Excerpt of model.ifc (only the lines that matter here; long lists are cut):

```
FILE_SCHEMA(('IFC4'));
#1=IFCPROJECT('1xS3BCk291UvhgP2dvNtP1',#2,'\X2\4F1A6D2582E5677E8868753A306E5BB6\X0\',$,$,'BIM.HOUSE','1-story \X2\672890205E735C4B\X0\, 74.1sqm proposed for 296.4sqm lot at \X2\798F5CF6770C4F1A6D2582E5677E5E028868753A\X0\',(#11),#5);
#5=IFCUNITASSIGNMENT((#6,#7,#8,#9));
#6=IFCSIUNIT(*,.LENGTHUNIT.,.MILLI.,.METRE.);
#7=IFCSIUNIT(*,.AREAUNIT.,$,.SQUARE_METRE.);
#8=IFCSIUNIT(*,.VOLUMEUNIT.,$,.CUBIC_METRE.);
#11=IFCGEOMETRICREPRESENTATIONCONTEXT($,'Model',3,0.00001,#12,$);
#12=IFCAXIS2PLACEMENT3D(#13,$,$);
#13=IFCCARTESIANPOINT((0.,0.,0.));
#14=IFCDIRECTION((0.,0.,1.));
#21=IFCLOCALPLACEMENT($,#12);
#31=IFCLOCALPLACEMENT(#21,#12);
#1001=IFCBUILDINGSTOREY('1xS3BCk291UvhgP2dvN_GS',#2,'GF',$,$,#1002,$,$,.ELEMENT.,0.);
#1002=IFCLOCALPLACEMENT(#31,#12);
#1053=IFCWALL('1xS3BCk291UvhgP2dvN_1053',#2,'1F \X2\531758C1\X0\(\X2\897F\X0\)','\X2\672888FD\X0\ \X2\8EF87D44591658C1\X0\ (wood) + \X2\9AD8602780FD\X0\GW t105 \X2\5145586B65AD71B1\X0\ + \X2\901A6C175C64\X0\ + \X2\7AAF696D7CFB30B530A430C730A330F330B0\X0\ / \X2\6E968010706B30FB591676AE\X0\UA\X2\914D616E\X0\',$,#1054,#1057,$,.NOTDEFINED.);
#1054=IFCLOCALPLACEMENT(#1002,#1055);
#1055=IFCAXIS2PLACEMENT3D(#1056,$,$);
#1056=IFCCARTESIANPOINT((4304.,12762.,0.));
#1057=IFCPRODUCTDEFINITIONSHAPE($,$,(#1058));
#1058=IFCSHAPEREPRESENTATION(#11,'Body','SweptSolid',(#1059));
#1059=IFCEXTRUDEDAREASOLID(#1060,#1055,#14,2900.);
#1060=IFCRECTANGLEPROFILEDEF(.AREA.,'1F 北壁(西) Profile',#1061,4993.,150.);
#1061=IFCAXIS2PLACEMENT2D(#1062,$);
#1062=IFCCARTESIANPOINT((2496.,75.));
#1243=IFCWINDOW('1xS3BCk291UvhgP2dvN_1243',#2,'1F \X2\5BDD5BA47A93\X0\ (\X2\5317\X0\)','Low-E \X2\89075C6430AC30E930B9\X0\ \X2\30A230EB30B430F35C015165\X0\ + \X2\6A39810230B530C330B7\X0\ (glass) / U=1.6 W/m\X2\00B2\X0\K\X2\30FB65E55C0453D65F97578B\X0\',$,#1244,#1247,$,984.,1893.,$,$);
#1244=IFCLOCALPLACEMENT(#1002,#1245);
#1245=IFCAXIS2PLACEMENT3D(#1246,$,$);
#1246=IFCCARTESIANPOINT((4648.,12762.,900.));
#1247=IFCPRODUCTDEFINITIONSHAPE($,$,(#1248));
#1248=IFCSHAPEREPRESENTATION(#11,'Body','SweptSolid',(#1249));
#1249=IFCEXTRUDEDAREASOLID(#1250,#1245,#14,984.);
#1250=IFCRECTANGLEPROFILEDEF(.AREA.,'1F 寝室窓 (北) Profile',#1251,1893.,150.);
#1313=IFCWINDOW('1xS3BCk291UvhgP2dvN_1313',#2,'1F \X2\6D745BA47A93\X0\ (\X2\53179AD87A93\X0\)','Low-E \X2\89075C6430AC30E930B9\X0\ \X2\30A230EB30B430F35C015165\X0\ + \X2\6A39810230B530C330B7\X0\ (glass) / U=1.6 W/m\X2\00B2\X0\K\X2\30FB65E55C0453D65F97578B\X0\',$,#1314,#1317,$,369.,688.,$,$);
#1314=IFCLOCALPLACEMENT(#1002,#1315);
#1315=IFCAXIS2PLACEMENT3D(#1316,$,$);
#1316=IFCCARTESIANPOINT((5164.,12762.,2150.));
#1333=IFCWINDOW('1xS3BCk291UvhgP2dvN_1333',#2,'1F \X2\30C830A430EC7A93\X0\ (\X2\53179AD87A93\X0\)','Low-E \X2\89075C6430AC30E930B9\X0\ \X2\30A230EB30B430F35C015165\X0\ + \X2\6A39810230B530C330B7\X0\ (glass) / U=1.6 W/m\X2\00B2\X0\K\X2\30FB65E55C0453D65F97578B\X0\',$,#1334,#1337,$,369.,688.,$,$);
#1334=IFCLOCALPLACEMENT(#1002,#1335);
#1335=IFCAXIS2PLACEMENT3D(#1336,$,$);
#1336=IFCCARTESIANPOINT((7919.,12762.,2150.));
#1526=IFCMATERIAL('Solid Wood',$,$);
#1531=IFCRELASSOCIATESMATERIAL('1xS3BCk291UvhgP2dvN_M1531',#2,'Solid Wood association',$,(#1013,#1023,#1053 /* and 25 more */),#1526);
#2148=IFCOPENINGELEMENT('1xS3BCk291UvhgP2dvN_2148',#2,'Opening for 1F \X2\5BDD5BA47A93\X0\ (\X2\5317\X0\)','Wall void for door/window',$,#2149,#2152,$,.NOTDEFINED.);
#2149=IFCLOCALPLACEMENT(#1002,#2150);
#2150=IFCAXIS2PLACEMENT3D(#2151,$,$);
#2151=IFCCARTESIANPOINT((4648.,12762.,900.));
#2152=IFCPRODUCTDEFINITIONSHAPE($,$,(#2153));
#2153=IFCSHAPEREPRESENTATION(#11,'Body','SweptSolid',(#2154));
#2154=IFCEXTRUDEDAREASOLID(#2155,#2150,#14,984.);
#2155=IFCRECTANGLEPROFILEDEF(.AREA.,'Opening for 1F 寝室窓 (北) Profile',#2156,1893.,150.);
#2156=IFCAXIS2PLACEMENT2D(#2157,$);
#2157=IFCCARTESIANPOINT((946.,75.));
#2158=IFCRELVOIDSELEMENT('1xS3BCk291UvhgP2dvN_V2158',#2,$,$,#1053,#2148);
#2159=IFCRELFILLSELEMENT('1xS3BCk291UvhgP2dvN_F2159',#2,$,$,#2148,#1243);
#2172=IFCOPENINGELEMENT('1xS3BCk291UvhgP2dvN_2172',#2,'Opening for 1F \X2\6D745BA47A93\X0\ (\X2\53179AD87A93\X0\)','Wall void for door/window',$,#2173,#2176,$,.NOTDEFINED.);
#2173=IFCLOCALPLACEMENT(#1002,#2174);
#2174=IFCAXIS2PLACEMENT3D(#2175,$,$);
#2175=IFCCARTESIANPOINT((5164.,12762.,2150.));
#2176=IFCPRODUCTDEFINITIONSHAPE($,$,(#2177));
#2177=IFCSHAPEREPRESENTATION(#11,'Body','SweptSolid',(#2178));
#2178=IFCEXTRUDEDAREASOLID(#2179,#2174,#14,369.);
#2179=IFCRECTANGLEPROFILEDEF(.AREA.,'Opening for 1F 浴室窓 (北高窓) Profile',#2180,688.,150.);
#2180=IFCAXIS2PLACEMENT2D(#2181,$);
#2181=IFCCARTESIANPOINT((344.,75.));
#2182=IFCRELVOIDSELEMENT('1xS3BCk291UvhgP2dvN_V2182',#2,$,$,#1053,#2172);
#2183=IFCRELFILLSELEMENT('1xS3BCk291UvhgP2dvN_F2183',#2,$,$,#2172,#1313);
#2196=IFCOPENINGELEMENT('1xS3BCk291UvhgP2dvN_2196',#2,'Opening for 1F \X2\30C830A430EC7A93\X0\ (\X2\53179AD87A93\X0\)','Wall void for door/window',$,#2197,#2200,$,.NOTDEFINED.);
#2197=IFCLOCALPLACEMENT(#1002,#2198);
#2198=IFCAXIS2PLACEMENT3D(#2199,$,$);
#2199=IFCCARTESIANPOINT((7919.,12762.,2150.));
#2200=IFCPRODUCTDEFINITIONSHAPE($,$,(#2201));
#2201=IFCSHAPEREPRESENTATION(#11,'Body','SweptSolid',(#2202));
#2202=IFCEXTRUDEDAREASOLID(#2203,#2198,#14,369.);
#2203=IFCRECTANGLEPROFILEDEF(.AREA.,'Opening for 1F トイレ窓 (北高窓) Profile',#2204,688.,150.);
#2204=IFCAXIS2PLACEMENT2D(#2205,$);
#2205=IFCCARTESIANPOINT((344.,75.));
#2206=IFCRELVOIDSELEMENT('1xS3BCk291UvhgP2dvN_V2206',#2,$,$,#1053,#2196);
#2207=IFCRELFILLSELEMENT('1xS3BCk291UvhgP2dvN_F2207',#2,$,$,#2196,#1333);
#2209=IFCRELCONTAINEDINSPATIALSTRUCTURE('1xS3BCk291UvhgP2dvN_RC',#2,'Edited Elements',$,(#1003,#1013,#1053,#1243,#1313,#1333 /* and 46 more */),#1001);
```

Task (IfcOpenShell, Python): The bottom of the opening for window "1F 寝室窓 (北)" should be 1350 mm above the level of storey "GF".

```python
import numpy as np
import ifcopenshell
import ifcopenshell.api.geometry
import ifcopenshell.geom
import ifcopenshell.util.element
import ifcopenshell.util.placement
import ifcopenshell.util.shape
import ifcopenshell.util.unit

model = ifcopenshell.open("model.ifc")
unit_scale = ifcopenshell.util.unit.calculate_unit_scale(model)

window = model.by_guid("1xS3BCk291UvhgP2dvN_1243")
opening = window.FillsVoids[0].RelatingOpeningElement
storey = ifcopenshell.util.element.get_container(window, ifc_class="IfcBuildingStorey")
level = ifcopenshell.util.placement.get_local_placement(storey.ObjectPlacement)[2, 3]

# The opening's origin need not be at the sill, so measure its lowest point.
shape = ifcopenshell.geom.create_shape(ifcopenshell.geom.settings(), opening)
bottom = ifcopenshell.util.shape.get_shape_bottom_elevation(shape, shape.geometry) / unit_scale
dz = level + 1.35 / unit_scale - bottom

shift = np.array([0.0, 0.0, dz])
# The window is not placed relative to its opening, so move both.
for product in (opening, window):
    matrix = ifcopenshell.util.placement.get_local_placement(product.ObjectPlacement)
    matrix[:3, 3] += shift
    ifcopenshell.api.geometry.edit_object_placement(model, product=product, matrix=matrix, is_si=False)

print(f"moved by {dz * unit_scale:+.3f} m")

model.write("model_updated.ifc")
```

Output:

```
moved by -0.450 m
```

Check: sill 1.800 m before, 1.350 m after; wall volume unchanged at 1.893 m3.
